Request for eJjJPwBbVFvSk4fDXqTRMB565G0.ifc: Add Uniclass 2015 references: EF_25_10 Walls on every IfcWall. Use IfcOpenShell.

First a look at what the model holds.

```python
import ifcopenshell

model = ifcopenshell.open("eJjJPwBbVFvSk4fDXqTRMB565G0.ifc")
print(model.schema)
print("classifications:", [c.Name for c in model.by_type("IfcClassification")])
for ifc_class in ("IfcDoor", "IfcRoof", "IfcStair", "IfcWall", "IfcWindow"):
    print(ifc_class, len(model.by_type(ifc_class)))
```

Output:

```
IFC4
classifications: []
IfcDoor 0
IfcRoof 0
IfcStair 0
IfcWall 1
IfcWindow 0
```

```python
import ifcopenshell
import ifcopenshell.api.classification

model = ifcopenshell.open("eJjJPwBbVFvSk4fDXqTRMB565G0.ifc")

system = ifcopenshell.api.classification.add_classification(model, classification="Uniclass 2015")

codes = {
    "IfcWall": ("EF_25_10", "Walls"),
}
for ifc_class, (code, name) in codes.items():
    products = model.by_type(ifc_class)
    ifcopenshell.api.classification.add_reference(
        model, products=products, classification=system, identification=code, name=name
    )
    print(code, len(products))

model.write("eJjJPwBbVFvSk4fDXqTRMB565G0-out.ifc")
```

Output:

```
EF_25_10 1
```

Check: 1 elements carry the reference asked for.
